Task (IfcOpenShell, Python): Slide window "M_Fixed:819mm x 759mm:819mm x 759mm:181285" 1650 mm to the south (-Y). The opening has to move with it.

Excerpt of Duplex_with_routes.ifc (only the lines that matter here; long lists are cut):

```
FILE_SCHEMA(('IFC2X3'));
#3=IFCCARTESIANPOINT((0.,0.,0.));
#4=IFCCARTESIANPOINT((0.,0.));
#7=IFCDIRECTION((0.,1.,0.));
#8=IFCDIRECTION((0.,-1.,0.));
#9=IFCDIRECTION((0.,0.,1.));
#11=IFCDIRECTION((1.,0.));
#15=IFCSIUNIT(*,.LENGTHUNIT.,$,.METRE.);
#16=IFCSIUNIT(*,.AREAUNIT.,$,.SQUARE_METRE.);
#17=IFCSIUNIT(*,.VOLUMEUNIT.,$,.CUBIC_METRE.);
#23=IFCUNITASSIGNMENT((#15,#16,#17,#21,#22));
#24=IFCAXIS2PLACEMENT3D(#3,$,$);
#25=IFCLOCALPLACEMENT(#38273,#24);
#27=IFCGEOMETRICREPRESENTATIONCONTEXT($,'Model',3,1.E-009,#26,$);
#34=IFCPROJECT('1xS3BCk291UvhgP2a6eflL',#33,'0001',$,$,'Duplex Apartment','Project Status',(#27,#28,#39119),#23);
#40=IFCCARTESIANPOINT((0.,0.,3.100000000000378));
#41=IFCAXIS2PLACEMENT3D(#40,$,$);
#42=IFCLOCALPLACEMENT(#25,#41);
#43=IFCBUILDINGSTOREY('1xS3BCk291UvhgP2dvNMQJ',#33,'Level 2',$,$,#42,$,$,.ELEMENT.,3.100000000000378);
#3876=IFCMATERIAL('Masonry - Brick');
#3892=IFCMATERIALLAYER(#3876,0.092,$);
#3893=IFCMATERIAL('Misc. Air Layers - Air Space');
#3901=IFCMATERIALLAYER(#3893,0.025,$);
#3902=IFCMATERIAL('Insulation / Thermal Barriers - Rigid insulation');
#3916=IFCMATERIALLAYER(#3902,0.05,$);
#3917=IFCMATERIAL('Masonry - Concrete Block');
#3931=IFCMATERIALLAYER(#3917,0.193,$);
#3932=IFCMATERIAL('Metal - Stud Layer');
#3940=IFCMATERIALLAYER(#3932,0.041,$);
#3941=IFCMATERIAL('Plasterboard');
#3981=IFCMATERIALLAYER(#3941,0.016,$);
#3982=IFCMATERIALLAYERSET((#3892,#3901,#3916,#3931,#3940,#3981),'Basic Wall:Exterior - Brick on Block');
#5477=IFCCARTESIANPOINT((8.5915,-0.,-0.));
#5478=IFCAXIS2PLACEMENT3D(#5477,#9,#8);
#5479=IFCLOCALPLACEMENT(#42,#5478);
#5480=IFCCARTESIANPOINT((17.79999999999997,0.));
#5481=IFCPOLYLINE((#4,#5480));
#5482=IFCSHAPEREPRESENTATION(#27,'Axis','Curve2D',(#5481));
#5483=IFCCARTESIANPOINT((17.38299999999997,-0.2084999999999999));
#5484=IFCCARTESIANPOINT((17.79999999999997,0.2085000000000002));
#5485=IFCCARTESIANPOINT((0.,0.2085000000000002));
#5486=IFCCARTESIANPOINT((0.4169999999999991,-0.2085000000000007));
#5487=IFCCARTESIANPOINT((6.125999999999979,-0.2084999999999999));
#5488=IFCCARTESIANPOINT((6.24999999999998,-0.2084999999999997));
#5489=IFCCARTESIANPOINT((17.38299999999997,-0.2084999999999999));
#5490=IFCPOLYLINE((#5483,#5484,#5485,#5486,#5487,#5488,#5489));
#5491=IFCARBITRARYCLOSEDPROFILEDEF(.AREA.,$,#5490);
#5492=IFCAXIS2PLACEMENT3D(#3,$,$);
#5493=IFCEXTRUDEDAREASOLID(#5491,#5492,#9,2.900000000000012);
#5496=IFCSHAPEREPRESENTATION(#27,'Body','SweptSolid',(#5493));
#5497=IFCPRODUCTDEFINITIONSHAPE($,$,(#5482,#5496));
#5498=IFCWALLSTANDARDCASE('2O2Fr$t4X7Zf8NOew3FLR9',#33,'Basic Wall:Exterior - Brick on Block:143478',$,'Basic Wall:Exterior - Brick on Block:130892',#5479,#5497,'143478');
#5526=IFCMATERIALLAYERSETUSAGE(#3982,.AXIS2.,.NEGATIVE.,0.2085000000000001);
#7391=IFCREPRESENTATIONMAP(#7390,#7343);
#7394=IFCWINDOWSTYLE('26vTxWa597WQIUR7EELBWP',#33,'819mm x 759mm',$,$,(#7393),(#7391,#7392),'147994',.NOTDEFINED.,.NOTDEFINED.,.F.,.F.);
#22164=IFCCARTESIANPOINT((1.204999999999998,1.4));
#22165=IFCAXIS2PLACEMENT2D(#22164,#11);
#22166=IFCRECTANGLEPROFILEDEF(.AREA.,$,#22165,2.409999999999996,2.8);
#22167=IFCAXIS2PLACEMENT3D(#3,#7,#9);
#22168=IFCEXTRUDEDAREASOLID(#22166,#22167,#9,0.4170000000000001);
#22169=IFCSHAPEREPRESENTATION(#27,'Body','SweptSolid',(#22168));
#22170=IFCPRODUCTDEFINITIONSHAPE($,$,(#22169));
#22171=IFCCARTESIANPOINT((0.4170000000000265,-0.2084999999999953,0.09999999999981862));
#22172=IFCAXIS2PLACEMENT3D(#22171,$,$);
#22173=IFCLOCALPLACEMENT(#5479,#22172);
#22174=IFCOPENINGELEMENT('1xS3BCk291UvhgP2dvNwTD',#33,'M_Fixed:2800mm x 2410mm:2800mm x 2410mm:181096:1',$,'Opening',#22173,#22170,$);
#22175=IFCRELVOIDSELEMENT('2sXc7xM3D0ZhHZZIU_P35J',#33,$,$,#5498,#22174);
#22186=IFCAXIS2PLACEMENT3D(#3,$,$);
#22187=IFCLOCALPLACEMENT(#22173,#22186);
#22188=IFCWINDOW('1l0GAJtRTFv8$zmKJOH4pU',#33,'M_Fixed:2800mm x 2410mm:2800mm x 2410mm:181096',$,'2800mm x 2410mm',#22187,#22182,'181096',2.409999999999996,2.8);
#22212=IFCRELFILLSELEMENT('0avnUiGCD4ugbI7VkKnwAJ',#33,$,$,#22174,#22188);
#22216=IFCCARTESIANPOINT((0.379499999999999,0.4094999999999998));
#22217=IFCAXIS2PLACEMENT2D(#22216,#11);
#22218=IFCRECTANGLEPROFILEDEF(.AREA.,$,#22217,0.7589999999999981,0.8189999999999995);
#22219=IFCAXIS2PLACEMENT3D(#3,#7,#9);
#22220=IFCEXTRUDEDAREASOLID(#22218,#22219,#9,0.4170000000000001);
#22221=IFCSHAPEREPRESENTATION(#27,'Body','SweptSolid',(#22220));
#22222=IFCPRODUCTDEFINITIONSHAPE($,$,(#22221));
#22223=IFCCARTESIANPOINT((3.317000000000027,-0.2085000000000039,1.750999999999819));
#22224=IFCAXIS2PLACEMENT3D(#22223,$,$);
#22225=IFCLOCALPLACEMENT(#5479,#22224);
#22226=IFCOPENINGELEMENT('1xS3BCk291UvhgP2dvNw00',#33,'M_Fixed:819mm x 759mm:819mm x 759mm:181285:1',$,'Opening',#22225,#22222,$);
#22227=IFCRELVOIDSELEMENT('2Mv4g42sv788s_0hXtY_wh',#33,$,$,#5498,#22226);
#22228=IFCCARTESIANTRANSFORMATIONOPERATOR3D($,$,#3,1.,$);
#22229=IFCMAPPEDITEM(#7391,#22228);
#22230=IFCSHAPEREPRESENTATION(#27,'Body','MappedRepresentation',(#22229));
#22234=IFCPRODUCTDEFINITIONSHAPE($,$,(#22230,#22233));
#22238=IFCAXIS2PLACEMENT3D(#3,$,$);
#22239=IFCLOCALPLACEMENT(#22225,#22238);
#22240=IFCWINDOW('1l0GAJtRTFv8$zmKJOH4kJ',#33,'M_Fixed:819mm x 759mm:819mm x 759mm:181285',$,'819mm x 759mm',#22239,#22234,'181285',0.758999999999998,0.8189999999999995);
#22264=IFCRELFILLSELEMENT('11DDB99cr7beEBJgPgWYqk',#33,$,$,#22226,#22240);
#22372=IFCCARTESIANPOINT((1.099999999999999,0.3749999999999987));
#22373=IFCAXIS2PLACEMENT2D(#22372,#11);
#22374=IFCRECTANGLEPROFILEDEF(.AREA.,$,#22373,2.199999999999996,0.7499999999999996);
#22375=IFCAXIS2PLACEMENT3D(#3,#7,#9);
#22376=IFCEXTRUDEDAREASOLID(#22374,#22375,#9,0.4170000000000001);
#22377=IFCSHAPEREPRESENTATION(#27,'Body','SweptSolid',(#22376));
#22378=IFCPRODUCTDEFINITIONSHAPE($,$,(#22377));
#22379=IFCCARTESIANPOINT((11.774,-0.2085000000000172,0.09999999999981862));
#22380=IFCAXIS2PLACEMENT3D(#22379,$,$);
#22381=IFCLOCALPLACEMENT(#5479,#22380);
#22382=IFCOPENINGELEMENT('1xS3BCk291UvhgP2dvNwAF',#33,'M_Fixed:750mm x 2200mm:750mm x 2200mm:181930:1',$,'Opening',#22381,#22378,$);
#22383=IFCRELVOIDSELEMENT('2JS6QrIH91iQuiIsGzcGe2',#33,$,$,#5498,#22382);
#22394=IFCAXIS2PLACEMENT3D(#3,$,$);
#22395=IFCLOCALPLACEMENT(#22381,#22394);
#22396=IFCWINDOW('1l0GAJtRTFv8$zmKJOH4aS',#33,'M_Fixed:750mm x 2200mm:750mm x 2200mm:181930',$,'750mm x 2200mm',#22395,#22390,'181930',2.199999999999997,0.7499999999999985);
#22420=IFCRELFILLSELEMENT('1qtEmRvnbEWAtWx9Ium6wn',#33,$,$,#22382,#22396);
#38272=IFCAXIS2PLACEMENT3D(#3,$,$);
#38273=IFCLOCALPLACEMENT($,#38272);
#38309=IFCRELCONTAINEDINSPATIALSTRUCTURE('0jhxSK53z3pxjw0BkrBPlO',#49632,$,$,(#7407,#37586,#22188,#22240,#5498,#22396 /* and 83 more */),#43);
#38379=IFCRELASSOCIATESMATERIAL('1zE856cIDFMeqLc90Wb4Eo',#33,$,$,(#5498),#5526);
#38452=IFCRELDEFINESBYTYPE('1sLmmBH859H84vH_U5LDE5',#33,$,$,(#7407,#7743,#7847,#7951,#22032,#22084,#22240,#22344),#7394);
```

```python
import ifcopenshell
import ifcopenshell.api.geometry
import ifcopenshell.util.placement
import ifcopenshell.util.unit

model = ifcopenshell.open("Duplex_with_routes.ifc")
unit_scale = ifcopenshell.util.unit.calculate_unit_scale(model)

window = model.by_guid("1l0GAJtRTFv8$zmKJOH4kJ")
opening = window.FillsVoids[0].RelatingOpeningElement
wall = opening.VoidsElements[0].RelatingBuildingElement

wall_matrix = ifcopenshell.util.placement.get_local_placement(wall.ObjectPlacement)
shift = wall_matrix[:3, 0] * 1.65 / unit_scale
before = ifcopenshell.util.placement.get_local_placement(window.ObjectPlacement)[:3, 3].copy()

# The window is placed relative to its opening, so it follows when the opening moves.
matrix = ifcopenshell.util.placement.get_local_placement(opening.ObjectPlacement)
matrix[:3, 3] += shift
ifcopenshell.api.geometry.edit_object_placement(
    model, product=opening, matrix=matrix, is_si=False, should_transform_children=True
)

after = ifcopenshell.util.placement.get_local_placement(window.ObjectPlacement)[:3, 3]
print("window moved by", (after - before).round(3) + 0.0)

model.write("Duplex_with_routes_updated.ifc")
```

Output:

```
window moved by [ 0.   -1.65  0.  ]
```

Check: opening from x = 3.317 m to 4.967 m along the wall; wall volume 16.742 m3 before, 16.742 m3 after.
